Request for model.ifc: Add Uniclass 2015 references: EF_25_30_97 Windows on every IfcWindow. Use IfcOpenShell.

First a look at what the model holds.

```python
import ifcopenshell

model = ifcopenshell.open("model.ifc")
print(model.schema)
print("classifications:", [c.Name for c in model.by_type("IfcClassification")])
for ifc_class in ("IfcDoor", "IfcRoof", "IfcStair", "IfcWall", "IfcWindow"):
    print(ifc_class, len(model.by_type(ifc_class)))
```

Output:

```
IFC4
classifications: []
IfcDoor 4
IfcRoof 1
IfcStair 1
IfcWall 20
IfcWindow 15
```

```python
import ifcopenshell
import ifcopenshell.api.classification

model = ifcopenshell.open("model.ifc")

system = ifcopenshell.api.classification.add_classification(model, classification="Uniclass 2015")

codes = {
    "IfcWindow": ("EF_25_30_97", "Windows"),
}
for ifc_class, (code, name) in codes.items():
    products = model.by_type(ifc_class)
    ifcopenshell.api.classification.add_reference(
        model, products=products, classification=system, identification=code, name=name
    )
    print(code, len(products))

model.write("model_v2.ifc")
```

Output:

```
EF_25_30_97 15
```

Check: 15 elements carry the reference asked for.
